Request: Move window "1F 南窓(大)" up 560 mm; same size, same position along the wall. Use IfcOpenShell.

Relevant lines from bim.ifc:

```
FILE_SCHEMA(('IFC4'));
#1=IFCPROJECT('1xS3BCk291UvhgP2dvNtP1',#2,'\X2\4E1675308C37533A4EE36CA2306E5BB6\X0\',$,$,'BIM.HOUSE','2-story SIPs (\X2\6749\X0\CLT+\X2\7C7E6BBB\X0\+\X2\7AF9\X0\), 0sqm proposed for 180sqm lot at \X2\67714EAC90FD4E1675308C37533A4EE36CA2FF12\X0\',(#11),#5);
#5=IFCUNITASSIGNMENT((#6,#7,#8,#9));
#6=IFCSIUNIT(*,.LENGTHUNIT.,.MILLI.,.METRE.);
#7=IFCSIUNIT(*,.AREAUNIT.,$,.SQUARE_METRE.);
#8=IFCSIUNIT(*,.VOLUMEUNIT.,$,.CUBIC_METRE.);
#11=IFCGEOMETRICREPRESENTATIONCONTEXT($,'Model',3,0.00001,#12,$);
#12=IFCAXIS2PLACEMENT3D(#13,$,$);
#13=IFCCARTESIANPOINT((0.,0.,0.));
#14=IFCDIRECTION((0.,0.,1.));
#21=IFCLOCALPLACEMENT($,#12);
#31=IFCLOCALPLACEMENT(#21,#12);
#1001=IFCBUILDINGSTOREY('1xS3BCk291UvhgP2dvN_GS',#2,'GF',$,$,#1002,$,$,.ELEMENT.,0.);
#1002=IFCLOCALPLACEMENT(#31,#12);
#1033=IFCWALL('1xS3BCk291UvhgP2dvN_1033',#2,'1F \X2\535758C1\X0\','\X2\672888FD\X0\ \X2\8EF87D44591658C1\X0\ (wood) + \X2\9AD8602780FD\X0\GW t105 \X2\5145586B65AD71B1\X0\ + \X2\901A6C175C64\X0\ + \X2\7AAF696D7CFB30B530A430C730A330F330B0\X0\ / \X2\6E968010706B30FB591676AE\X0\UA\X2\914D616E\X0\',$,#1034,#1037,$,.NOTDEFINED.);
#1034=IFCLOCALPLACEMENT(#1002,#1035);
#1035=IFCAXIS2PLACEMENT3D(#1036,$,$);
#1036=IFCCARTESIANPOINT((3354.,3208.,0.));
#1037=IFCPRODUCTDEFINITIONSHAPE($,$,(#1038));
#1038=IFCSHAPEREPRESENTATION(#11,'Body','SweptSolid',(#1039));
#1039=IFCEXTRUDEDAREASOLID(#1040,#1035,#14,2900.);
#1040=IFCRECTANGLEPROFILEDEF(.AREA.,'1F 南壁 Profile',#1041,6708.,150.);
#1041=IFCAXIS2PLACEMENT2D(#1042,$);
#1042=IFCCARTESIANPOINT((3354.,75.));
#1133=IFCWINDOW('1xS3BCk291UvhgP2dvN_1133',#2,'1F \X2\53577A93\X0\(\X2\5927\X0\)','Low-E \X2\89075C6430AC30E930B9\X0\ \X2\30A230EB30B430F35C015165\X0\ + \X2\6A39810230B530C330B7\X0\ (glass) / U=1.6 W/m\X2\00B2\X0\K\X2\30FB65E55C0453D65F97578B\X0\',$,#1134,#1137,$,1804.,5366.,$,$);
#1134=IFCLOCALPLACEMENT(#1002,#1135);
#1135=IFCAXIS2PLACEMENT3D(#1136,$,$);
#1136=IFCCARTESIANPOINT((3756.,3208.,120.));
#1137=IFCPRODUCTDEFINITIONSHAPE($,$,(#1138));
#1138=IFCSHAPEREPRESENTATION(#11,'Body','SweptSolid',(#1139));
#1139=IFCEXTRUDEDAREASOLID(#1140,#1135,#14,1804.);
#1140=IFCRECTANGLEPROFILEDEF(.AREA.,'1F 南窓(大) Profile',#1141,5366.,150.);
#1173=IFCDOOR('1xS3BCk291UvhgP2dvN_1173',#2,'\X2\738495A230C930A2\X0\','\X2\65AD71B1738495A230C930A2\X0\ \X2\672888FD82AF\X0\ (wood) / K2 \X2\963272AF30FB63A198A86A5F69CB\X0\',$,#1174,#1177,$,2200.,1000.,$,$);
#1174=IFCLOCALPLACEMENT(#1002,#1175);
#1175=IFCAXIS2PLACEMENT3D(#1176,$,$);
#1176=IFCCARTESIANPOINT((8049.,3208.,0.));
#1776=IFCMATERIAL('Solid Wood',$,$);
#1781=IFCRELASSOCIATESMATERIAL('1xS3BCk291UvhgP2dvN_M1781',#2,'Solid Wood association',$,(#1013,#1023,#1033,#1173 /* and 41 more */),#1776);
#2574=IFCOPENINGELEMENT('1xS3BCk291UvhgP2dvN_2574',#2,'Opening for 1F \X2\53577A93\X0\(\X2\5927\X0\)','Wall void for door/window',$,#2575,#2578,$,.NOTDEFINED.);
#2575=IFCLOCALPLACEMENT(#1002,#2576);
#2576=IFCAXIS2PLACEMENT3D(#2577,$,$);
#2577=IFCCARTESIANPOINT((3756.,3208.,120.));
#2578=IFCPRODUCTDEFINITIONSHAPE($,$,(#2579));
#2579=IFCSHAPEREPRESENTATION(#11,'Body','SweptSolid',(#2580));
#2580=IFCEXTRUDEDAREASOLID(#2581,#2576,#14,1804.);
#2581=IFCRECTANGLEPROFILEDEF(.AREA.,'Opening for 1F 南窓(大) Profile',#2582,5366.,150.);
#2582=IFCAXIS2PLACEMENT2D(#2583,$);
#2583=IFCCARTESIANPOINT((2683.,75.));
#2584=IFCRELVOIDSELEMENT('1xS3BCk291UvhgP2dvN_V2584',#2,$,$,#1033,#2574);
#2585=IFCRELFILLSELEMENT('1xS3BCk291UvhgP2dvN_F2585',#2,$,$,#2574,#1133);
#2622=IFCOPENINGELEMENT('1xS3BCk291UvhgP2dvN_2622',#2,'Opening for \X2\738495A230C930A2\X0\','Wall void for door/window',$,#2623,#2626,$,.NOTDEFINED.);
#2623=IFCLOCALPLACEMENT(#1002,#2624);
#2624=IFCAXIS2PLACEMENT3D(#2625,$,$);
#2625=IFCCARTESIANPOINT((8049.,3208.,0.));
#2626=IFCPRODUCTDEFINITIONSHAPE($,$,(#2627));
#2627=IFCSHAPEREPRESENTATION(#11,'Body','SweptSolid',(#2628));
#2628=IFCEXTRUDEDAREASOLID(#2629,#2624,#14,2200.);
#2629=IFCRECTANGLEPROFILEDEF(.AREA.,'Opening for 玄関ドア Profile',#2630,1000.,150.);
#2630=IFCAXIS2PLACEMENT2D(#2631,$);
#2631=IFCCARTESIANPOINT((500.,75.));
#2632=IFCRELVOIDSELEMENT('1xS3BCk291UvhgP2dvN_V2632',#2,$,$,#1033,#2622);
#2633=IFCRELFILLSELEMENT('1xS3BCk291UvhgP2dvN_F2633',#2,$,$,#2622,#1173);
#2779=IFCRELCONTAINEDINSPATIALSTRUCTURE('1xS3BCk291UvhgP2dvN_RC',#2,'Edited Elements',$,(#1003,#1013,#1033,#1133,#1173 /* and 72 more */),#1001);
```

```python
import numpy as np
import ifcopenshell
import ifcopenshell.api.geometry
import ifcopenshell.util.placement
import ifcopenshell.util.unit

model = ifcopenshell.open("bim.ifc")
unit_scale = ifcopenshell.util.unit.calculate_unit_scale(model)

window = model.by_id(1133)
opening = window.FillsVoids[0].RelatingOpeningElement
dz = 0.56 / unit_scale

shift = np.array([0.0, 0.0, dz])
# The window is not placed relative to its opening, so move both.
for product in (opening, window):
    matrix = ifcopenshell.util.placement.get_local_placement(product.ObjectPlacement)
    matrix[:3, 3] += shift
    ifcopenshell.api.geometry.edit_object_placement(model, product=product, matrix=matrix, is_si=False)

print(f"moved by {dz * unit_scale:+.3f} m")

model.write("bim_edited.ifc")
```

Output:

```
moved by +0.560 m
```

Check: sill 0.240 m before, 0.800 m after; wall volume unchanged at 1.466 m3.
